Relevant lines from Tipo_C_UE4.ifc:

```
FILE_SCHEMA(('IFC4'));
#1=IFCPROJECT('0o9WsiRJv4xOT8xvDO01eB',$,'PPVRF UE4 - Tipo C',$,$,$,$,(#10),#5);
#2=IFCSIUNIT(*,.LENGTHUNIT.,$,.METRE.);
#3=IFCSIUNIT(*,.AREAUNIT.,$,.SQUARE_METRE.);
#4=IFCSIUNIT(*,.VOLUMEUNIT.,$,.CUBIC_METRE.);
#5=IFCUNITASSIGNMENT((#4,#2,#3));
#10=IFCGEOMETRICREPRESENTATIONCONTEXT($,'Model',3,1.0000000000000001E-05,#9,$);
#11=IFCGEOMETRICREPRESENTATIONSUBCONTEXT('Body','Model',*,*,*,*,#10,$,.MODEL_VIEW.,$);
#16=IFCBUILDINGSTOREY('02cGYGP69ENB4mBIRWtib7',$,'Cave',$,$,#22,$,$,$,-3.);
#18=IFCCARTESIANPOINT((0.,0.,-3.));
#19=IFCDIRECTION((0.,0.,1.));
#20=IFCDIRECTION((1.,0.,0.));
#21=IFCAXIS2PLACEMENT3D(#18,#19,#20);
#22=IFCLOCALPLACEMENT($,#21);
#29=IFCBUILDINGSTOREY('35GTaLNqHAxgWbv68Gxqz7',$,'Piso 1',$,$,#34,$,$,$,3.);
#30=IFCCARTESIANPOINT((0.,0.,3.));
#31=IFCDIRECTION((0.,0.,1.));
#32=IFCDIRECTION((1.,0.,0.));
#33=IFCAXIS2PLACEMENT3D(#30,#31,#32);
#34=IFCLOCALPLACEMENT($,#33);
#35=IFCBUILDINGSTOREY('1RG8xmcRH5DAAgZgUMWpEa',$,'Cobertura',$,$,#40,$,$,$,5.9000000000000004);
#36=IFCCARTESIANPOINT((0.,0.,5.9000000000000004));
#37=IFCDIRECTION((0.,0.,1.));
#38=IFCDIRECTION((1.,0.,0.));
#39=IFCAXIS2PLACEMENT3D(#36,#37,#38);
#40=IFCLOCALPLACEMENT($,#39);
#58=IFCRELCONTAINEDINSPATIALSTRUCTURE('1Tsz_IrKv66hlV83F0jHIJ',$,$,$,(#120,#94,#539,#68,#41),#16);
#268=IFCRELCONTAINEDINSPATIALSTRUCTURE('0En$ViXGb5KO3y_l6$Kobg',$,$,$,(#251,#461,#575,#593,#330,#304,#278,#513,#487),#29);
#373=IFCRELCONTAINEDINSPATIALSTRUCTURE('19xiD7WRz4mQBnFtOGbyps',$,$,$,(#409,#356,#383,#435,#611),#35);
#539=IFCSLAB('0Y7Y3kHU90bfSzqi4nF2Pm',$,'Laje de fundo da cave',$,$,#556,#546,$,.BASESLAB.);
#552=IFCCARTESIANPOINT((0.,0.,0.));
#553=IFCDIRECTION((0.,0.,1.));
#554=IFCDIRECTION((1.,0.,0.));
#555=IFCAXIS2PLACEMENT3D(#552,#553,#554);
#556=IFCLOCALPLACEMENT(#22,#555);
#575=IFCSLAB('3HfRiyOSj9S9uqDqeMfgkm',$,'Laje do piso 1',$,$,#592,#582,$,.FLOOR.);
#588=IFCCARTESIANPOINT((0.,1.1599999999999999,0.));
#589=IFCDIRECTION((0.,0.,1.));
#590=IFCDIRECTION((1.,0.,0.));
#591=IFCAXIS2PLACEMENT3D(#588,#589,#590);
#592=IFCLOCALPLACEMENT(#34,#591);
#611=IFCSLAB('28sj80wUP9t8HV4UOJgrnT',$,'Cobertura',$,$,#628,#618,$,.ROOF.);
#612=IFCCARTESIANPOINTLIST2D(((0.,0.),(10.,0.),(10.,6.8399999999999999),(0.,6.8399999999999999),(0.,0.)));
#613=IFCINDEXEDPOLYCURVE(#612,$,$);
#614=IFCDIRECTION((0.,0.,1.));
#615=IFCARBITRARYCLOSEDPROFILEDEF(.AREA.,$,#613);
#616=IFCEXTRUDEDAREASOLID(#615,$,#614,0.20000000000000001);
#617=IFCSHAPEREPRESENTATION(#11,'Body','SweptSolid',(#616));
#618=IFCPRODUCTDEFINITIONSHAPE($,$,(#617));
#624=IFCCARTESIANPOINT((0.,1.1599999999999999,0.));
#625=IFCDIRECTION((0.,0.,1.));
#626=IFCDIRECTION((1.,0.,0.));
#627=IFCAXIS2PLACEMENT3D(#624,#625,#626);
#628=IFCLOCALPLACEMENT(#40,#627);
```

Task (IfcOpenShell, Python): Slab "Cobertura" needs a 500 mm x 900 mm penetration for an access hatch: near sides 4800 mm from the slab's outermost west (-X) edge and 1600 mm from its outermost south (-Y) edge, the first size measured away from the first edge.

```python
import numpy as np
import ifcopenshell
import ifcopenshell.api.feature
import ifcopenshell.api.geometry
import ifcopenshell.api.root
import ifcopenshell.geom
import ifcopenshell.util.placement
import ifcopenshell.util.representation
import ifcopenshell.util.shape
import ifcopenshell.util.unit

model = ifcopenshell.open("Tipo_C_UE4.ifc")
unit_scale = ifcopenshell.util.unit.calculate_unit_scale(model)
settings = ifcopenshell.geom.settings()


def volume(element):
    """Net volume in cubic metres, openings subtracted."""
    shape = ifcopenshell.geom.create_shape(settings, element)
    return ifcopenshell.util.shape.get_volume(shape.geometry)


slab = model.by_guid("28sj80wUP9t8HV4UOJgrnT")
before = volume(slab)

# Extent in the slab's own axes, in metres. The edges named are its -X and -Y sides.
slab_shape = ifcopenshell.geom.create_shape(settings, slab)
vertices = ifcopenshell.util.shape.get_vertices(slab_shape.geometry)
x_min, y_min, bottom = vertices.min(axis=0)
top = vertices[:, 2].max()

opening = ifcopenshell.api.root.create_entity(model, ifc_class="IfcOpeningElement", name="Access hatch opening", predefined_type="OPENING")
context = ifcopenshell.util.representation.get_context(model, "Model", "Body", "MODEL_VIEW")
width, depth = 0.5, 0.9
outline = [(0.0, 0.0), (width, 0.0), (width, depth), (0.0, depth), (0.0, 0.0)]
# Overshoot both faces by 50 mm so the cut is clean.
shape = ifcopenshell.api.geometry.add_slab_representation(
    model, context=context, depth=top - bottom + 0.1, polyline=outline
)
ifcopenshell.api.geometry.assign_representation(model, product=opening, representation=shape)

matrix = ifcopenshell.util.placement.get_local_placement(slab.ObjectPlacement)
matrix[:, 3] = matrix @ np.append(np.array([x_min + 4.8, y_min + 1.6, bottom - 0.05]) / unit_scale, 1.0)
ifcopenshell.api.geometry.edit_object_placement(model, product=opening, matrix=matrix, is_si=False)
ifcopenshell.api.feature.add_feature(model, feature=opening, element=slab)

after = volume(slab)

print(f"slab volume {before:.3f} -> {after:.3f} m3")

model.write("Tipo_C_UE4_v2.ifc")
```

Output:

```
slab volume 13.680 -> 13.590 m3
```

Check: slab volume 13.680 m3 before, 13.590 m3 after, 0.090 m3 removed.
